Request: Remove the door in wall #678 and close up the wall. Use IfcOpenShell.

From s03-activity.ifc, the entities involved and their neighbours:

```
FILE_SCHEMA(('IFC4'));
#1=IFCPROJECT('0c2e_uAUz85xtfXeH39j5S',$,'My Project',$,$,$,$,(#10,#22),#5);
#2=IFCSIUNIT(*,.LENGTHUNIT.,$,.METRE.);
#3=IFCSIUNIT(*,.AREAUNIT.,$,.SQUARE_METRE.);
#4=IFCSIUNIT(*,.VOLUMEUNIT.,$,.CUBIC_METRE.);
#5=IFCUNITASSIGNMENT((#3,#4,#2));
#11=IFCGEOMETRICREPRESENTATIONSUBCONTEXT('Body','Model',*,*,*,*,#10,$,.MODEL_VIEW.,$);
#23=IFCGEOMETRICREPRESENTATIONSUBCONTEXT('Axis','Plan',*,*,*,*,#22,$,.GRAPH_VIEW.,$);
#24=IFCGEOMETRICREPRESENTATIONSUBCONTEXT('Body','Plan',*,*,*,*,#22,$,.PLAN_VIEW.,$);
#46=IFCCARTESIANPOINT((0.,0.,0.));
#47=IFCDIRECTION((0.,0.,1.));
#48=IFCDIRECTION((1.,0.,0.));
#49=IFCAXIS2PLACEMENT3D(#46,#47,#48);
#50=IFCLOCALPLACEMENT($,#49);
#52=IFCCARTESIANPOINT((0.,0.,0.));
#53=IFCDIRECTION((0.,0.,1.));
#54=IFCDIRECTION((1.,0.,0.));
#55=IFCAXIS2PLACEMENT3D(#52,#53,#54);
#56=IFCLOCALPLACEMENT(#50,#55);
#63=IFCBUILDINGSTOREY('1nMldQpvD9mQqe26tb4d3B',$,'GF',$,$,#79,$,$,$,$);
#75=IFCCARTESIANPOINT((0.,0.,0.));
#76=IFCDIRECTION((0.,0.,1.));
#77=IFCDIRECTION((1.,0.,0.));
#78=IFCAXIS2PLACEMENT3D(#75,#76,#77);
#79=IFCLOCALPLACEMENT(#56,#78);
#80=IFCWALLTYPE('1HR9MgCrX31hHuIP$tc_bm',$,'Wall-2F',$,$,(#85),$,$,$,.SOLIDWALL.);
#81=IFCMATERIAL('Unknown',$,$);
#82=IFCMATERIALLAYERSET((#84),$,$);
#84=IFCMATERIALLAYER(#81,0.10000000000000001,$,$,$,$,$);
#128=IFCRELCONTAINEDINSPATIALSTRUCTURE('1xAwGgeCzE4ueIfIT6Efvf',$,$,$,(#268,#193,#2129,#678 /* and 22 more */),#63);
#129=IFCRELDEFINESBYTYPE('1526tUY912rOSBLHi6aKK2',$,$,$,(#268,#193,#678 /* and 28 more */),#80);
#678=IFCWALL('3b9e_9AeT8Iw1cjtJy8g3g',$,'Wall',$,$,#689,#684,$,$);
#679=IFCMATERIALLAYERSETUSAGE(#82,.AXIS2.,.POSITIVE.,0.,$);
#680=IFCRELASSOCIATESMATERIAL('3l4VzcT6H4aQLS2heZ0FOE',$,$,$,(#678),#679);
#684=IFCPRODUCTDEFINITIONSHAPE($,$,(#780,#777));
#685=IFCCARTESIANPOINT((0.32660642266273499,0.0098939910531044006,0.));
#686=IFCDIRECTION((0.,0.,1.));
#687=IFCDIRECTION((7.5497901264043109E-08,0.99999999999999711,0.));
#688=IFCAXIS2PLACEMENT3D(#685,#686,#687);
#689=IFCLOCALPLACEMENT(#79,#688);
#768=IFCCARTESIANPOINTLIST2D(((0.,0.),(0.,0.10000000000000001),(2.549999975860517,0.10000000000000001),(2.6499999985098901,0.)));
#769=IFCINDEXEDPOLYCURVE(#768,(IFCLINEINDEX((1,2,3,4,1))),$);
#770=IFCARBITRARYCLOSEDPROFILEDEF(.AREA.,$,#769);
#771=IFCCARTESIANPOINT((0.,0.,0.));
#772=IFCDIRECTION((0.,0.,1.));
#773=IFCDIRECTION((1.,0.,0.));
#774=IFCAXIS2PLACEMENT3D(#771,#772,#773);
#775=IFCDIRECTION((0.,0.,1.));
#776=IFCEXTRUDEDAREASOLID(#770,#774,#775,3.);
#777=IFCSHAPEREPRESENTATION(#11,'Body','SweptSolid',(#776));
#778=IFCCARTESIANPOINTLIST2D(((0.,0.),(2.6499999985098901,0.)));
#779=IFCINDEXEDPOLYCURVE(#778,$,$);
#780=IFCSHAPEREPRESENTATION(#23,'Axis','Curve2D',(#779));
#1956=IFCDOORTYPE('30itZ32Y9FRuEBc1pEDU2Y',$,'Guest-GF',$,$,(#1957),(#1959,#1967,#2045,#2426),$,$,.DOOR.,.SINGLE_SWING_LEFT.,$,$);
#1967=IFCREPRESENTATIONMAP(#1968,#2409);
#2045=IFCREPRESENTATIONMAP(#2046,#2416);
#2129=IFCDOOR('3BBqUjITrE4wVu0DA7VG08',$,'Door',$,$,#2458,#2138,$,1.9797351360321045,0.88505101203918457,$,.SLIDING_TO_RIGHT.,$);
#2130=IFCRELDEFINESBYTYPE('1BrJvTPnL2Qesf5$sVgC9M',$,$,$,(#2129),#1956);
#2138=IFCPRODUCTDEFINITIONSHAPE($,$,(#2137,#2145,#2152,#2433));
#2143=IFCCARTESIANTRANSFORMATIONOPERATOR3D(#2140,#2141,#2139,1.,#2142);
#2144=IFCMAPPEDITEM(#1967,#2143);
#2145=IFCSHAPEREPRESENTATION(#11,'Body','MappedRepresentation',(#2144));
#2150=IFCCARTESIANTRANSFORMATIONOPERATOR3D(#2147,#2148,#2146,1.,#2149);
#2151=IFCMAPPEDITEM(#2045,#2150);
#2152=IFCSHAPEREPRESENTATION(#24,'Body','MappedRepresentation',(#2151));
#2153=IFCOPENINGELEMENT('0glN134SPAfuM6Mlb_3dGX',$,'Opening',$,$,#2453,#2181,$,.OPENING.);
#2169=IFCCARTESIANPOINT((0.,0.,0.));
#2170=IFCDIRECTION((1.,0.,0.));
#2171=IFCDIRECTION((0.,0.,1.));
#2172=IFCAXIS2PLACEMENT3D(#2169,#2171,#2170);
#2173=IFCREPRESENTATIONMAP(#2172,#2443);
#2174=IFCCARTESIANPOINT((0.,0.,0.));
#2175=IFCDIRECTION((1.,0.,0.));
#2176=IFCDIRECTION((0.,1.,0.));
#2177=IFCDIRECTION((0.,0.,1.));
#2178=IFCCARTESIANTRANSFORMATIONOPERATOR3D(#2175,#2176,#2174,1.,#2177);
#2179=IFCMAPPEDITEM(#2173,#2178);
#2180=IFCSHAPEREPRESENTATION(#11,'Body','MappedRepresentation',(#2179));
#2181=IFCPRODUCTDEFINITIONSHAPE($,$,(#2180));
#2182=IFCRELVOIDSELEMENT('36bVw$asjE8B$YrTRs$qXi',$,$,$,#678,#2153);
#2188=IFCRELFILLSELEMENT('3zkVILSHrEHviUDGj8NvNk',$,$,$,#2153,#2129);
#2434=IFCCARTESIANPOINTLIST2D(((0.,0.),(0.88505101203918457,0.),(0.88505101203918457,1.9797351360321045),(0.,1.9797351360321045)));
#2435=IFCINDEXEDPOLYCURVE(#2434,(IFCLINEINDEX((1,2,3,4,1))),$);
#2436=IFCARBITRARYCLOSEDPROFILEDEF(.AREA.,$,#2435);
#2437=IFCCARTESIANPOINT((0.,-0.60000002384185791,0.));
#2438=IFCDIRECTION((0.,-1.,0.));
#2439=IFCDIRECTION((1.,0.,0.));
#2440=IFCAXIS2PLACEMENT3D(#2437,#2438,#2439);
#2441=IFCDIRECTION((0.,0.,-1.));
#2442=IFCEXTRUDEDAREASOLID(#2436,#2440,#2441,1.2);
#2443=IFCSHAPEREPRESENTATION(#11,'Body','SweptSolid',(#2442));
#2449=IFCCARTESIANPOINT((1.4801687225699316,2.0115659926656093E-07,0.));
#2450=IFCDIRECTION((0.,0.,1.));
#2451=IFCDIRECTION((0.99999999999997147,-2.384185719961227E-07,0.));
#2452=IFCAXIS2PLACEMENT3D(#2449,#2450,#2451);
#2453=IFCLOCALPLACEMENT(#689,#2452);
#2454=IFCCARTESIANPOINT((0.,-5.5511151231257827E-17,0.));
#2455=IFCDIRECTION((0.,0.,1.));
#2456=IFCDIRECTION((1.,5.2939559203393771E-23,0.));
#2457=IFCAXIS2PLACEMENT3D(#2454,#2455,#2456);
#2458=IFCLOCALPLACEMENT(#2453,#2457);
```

```python
import ifcopenshell
import ifcopenshell.api.feature
import ifcopenshell.api.root
import ifcopenshell.geom
import ifcopenshell.util.shape

model = ifcopenshell.open("s03-activity.ifc")
settings = ifcopenshell.geom.settings()


def volume(element):
    """Net volume in cubic metres, openings subtracted."""
    shape = ifcopenshell.geom.create_shape(settings, element)
    return ifcopenshell.util.shape.get_volume(shape.geometry)


door = model.by_guid("3BBqUjITrE4wVu0DA7VG08")
opening = door.FillsVoids[0].RelatingOpeningElement
wall = opening.VoidsElements[0].RelatingBuildingElement
before = volume(wall)

ifcopenshell.api.root.remove_product(model, product=door)
ifcopenshell.api.feature.remove_feature(model, feature=opening)

after = volume(wall)

print(f"wall volume {before:.3f} -> {after:.3f} m3")

model.write("s03-activity_v2.ifc")
```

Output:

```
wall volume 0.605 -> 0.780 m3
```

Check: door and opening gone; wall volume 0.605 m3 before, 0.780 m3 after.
